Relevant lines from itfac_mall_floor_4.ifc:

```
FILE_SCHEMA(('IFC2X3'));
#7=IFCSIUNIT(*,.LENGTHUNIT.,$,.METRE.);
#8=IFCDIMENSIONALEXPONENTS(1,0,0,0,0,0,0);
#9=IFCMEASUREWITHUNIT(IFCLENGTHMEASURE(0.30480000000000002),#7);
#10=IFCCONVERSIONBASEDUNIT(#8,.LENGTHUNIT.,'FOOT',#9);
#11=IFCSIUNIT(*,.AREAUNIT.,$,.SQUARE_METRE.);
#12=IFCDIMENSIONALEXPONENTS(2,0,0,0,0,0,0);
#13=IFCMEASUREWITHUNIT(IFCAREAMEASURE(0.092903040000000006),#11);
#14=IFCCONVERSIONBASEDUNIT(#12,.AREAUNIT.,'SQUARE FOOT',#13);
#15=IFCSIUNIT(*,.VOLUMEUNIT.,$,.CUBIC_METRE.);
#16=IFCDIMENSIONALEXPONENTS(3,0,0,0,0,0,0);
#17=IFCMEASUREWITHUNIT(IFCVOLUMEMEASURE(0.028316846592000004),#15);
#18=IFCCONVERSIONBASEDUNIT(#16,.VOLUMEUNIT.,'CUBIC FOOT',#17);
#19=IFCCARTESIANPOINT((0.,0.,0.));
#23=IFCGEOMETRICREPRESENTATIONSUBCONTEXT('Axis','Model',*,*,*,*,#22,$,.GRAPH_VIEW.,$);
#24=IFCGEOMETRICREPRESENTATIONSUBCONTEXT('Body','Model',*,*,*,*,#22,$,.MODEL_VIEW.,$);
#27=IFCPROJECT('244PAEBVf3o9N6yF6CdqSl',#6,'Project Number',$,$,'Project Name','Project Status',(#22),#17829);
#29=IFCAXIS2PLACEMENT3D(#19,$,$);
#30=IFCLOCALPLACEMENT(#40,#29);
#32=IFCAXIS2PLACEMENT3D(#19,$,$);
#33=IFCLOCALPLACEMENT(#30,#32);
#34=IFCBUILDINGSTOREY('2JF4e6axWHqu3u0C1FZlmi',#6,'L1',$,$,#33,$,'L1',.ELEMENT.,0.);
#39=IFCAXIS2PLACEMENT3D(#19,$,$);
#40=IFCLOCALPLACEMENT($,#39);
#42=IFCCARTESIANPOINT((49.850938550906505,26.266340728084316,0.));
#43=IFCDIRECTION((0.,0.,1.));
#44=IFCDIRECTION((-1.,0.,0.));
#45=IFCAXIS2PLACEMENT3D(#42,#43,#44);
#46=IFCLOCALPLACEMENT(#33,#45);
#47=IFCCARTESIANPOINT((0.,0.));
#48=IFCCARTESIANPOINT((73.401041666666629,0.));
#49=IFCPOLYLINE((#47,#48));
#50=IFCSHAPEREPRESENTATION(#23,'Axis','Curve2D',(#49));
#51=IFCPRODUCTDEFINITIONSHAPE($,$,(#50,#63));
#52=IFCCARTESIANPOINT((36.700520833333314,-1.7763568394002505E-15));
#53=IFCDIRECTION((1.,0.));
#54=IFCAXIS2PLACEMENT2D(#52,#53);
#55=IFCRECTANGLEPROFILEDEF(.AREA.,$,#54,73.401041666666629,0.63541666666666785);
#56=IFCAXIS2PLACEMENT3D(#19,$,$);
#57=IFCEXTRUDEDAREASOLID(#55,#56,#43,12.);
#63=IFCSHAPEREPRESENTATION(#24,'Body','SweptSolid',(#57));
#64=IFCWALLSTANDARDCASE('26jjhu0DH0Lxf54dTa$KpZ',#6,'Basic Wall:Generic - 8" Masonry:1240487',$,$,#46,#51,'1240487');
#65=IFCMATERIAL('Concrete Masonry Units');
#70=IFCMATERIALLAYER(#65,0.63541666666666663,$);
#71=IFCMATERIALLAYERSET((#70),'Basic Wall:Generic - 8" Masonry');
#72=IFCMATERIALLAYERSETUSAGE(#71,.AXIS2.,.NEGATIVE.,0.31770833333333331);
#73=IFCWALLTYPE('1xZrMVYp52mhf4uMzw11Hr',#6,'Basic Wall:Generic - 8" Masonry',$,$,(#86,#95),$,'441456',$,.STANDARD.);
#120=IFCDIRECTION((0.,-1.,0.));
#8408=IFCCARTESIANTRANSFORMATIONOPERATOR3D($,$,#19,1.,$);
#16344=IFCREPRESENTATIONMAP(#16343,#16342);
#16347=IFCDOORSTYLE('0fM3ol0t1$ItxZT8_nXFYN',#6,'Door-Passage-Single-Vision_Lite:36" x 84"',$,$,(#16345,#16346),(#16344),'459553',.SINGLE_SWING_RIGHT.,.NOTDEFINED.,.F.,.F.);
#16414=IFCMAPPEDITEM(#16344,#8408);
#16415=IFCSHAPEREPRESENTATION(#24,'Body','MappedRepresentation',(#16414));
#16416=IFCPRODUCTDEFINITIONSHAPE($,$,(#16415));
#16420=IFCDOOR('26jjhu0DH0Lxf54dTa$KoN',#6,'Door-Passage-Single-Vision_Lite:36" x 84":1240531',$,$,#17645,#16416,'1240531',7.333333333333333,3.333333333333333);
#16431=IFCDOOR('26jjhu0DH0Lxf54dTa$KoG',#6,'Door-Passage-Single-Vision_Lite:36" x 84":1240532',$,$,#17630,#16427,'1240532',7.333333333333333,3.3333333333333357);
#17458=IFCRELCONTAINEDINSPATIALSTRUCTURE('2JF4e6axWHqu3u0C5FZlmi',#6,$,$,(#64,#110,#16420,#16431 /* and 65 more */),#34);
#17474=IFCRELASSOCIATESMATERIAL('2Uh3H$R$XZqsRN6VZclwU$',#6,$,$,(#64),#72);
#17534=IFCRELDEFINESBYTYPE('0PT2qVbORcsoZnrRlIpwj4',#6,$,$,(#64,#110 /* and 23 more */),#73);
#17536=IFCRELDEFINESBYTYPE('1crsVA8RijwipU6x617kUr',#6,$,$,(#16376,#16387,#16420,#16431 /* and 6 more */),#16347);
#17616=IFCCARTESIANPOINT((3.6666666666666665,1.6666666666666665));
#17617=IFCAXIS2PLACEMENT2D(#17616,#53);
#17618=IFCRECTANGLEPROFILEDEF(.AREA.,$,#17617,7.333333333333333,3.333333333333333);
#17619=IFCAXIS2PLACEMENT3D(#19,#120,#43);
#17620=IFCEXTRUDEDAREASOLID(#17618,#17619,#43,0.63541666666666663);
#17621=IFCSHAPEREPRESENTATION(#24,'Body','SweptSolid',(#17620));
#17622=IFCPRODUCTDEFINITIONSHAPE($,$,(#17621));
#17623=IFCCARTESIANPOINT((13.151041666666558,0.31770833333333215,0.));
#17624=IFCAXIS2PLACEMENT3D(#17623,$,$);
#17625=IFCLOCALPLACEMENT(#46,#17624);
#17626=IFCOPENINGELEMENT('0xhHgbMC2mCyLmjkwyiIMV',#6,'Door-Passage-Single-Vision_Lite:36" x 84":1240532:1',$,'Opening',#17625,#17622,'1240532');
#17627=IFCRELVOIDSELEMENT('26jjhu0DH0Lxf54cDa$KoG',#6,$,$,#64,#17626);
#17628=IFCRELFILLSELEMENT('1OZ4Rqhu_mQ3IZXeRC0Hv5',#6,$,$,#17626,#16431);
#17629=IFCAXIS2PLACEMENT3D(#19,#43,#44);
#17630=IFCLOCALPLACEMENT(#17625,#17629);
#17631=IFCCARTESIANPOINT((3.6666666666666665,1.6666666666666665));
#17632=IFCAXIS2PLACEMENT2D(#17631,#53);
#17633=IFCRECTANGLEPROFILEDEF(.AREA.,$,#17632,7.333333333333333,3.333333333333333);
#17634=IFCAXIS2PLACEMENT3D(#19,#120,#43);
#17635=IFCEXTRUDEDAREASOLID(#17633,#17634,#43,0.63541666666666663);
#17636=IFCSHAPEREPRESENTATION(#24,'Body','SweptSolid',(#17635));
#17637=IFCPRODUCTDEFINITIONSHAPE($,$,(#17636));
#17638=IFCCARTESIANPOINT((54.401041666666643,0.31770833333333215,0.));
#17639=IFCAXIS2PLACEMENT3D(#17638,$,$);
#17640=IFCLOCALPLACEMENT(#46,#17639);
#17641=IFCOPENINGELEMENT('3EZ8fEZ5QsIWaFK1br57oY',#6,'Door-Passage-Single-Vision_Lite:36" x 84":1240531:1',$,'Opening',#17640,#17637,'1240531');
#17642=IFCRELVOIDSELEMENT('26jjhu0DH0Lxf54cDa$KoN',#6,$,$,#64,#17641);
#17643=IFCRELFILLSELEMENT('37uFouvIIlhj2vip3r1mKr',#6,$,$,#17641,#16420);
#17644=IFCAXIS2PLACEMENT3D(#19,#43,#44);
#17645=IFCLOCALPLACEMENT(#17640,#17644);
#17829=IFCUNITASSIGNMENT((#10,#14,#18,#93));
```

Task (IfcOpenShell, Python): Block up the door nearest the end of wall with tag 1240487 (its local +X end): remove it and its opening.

```python
import ifcopenshell
import ifcopenshell.api.feature
import ifcopenshell.api.root
import ifcopenshell.geom
import ifcopenshell.util.shape

model = ifcopenshell.open("itfac_mall_floor_4.ifc")
settings = ifcopenshell.geom.settings()


def volume(element):
    """Net volume in cubic metres, openings subtracted."""
    shape = ifcopenshell.geom.create_shape(settings, element)
    return ifcopenshell.util.shape.get_volume(shape.geometry)


door = model.by_guid("26jjhu0DH0Lxf54dTa$KoN")
opening = door.FillsVoids[0].RelatingOpeningElement
wall = opening.VoidsElements[0].RelatingBuildingElement
before = volume(wall)

ifcopenshell.api.root.remove_product(model, product=door)
ifcopenshell.api.feature.remove_feature(model, feature=opening)

after = volume(wall)

print(f"wall volume {before:.3f} -> {after:.3f} m3")

model.write("itfac_mall_floor_4_edited.ifc")
```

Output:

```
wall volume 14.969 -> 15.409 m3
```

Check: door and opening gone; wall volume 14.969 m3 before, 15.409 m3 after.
